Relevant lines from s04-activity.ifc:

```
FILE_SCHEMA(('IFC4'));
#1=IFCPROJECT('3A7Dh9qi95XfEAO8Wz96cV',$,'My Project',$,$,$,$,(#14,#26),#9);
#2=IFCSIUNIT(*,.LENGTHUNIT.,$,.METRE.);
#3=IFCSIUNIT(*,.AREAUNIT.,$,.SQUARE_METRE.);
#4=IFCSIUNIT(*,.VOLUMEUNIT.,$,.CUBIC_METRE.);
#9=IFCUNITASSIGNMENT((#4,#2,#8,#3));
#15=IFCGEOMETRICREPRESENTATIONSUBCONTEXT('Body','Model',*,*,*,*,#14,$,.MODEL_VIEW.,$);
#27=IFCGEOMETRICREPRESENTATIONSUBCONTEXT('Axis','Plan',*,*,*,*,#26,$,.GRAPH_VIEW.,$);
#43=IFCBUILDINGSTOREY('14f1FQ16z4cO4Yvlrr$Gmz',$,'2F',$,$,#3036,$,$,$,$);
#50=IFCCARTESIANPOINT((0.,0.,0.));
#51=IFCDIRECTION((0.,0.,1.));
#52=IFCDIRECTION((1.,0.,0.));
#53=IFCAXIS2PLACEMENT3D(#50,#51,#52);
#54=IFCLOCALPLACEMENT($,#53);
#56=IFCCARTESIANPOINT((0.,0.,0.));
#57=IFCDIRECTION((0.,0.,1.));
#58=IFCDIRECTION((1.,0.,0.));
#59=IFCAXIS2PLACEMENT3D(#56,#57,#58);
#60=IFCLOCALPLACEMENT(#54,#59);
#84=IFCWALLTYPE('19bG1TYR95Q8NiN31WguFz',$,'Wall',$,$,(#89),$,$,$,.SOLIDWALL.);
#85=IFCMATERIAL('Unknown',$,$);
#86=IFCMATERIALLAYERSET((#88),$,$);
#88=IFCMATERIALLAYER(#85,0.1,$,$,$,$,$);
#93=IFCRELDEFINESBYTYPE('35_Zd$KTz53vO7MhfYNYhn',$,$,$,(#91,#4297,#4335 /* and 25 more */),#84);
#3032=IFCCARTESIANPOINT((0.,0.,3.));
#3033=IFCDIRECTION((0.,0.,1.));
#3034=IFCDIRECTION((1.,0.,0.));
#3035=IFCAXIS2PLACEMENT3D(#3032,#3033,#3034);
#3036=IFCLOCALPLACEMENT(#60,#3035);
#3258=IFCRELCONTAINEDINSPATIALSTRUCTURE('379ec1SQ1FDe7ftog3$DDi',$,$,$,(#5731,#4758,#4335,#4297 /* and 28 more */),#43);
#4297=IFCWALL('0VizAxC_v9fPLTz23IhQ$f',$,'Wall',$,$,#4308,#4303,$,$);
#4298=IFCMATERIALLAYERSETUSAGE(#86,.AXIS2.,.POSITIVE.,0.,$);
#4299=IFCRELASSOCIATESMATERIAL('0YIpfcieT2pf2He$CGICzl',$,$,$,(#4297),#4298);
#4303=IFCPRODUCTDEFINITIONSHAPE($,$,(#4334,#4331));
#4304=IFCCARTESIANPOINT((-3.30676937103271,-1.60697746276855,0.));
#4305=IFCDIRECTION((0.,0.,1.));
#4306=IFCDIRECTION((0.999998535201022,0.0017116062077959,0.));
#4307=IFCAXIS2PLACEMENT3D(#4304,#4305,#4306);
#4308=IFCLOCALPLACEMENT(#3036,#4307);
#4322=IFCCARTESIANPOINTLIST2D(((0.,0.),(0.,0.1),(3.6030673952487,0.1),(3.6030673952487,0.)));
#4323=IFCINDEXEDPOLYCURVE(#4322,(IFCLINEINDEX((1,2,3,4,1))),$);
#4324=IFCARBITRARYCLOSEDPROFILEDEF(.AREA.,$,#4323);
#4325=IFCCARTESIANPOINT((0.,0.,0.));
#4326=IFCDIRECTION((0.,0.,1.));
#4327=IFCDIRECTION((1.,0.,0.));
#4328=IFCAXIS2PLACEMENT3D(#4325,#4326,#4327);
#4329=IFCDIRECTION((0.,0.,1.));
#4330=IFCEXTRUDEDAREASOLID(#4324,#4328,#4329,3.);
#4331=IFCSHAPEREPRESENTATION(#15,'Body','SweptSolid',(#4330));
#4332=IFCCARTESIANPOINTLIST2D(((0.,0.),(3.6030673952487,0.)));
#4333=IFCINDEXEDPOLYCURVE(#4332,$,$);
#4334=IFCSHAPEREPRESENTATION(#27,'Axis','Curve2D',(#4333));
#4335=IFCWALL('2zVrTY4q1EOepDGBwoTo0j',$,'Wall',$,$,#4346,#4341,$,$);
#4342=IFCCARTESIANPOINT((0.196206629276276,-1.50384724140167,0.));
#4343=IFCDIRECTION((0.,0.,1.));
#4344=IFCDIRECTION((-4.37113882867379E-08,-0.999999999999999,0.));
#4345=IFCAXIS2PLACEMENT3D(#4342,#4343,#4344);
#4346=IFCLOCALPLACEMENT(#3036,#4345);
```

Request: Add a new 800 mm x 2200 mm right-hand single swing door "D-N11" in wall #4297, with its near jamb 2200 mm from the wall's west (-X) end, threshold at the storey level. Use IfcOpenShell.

```python
import numpy as np
import ifcopenshell
import ifcopenshell.api.feature
import ifcopenshell.api.geometry
import ifcopenshell.api.root
import ifcopenshell.api.spatial
import ifcopenshell.geom
import ifcopenshell.util.element
import ifcopenshell.util.placement
import ifcopenshell.util.representation
import ifcopenshell.util.shape
import ifcopenshell.util.unit

model = ifcopenshell.open("s04-activity.ifc")
unit_scale = ifcopenshell.util.unit.calculate_unit_scale(model)
settings = ifcopenshell.geom.settings()


def volume(element):
    """Net volume in cubic metres, openings subtracted."""
    shape = ifcopenshell.geom.create_shape(settings, element)
    return ifcopenshell.util.shape.get_volume(shape.geometry)


wall = model.by_guid("0VizAxC_v9fPLTz23IhQ$f")
storey = ifcopenshell.util.element.get_container(wall, ifc_class="IfcBuildingStorey")
context = ifcopenshell.util.representation.get_context(model, "Model", "Body", "MODEL_VIEW")
before = volume(wall)

width, height, from_end, sill = 0.8, 2.2, 2.2, 0.0  # metres

# The wall runs along its own X axis, and the end named is its -X end.
wall_shape = ifcopenshell.geom.create_shape(settings, wall)
x, y, z = ifcopenshell.util.shape.get_vertices(wall_shape.geometry).T
start = x.min() + from_end
face, thickness = float(y.min()), float(y.max() - y.min())
wall_matrix = ifcopenshell.util.placement.get_local_placement(wall.ObjectPlacement)
level = ifcopenshell.util.placement.get_local_placement(storey.ObjectPlacement)[2, 3]


def in_wall(x, y):
    """Placement at x, y metres in the wall's axes, at sill height."""
    matrix = wall_matrix.copy()
    matrix[:, 3] = wall_matrix @ np.array([x / unit_scale, y / unit_scale, 0.0, 1.0])
    matrix[2, 3] = level + sill / unit_scale
    return matrix


# Opening: a box that overshoots both wall faces by 50 mm.
opening = ifcopenshell.api.root.create_entity(model, ifc_class="IfcOpeningElement", predefined_type="OPENING")
box = ifcopenshell.api.geometry.add_wall_representation(
    model, context=context, length=width, height=height, thickness=thickness + 0.1
)
ifcopenshell.api.geometry.assign_representation(model, product=opening, representation=box)
ifcopenshell.api.geometry.edit_object_placement(model, product=opening, matrix=in_wall(start, face - 0.05), is_si=False)
ifcopenshell.api.feature.add_feature(model, feature=opening, element=wall)

door = ifcopenshell.api.root.create_entity(model, ifc_class="IfcDoor", name="D-N11", predefined_type="DOOR")
door.OverallWidth, door.OverallHeight = width / unit_scale, height / unit_scale
door.OperationType = "SINGLE_SWING_RIGHT"
body = ifcopenshell.api.geometry.add_door_representation(
    model,
    context=context,
    overall_width=door.OverallWidth,
    overall_height=door.OverallHeight,
    operation_type="SINGLE_SWING_RIGHT",
    lining_properties={"LiningDepth": thickness / unit_scale, "ThresholdDepth": thickness / unit_scale},
)
ifcopenshell.api.geometry.assign_representation(model, product=door, representation=body)
ifcopenshell.api.spatial.assign_container(model, products=[door], relating_structure=storey)
ifcopenshell.api.feature.add_filling(model, opening=opening, element=door)

# The lining spans the wall, so the door starts at the wall face.
ifcopenshell.api.geometry.edit_object_placement(model, product=door, matrix=in_wall(start, face), is_si=False)

after = volume(wall)

print(f"wall volume {before:.3f} -> {after:.3f} m3")

model.write("s04-activity-out.ifc")
```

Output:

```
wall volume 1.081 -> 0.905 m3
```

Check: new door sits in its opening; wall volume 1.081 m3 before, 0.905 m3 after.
